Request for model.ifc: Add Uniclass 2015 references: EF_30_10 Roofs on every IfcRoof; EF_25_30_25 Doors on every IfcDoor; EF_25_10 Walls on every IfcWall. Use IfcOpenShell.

First a look at what the model holds.

```python
import ifcopenshell

model = ifcopenshell.open("model.ifc")
print(model.schema)
print("classifications:", [c.Name for c in model.by_type("IfcClassification")])
for ifc_class in ("IfcDoor", "IfcRoof", "IfcStair", "IfcWall", "IfcWindow"):
    print(ifc_class, len(model.by_type(ifc_class)))
```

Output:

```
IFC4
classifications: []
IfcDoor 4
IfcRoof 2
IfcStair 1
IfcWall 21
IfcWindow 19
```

```python
import ifcopenshell
import ifcopenshell.api.classification

model = ifcopenshell.open("model.ifc")

system = ifcopenshell.api.classification.add_classification(model, classification="Uniclass 2015")

codes = {
    "IfcRoof": ("EF_30_10", "Roofs"),
    "IfcDoor": ("EF_25_30_25", "Doors"),
    "IfcWall": ("EF_25_10", "Walls"),
}
for ifc_class, (code, name) in codes.items():
    products = model.by_type(ifc_class)
    ifcopenshell.api.classification.add_reference(
        model, products=products, classification=system, identification=code, name=name
    )
    print(code, len(products))

model.write("model_rev.ifc")
```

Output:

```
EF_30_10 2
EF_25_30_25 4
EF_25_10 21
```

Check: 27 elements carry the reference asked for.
